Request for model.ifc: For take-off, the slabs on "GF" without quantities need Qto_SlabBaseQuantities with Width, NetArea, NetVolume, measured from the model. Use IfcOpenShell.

First a look at what the model holds.

```python
import ifcopenshell
import ifcopenshell.util.element
import ifcopenshell.util.unit

model = ifcopenshell.open("model.ifc")
print(model.schema)
for unit_type in ("LENGTHUNIT", "AREAUNIT", "VOLUMEUNIT"):
    print(unit_type, ifcopenshell.util.unit.calculate_unit_scale(model, unit_type))
storey = next(s for s in model.by_type("IfcBuildingStorey") if s.Name == "GF")
slabs = [e for e in ifcopenshell.util.element.get_decomposition(storey) if e.is_a("IfcSlab")]
for e in sorted(slabs, key=lambda e: e.id()):
    print(e.id(), e.is_a(), e.Name, list(ifcopenshell.util.element.get_psets(e, qtos_only=True)), sep=" | ")
```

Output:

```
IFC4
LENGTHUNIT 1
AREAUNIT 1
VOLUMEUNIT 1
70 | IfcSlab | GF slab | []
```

```python
import ifcopenshell
import ifcopenshell.api.pset
import ifcopenshell.geom
import ifcopenshell.util.element
import ifcopenshell.util.shape
import ifcopenshell.util.unit

model = ifcopenshell.open("model.ifc")
unit_scale = ifcopenshell.util.unit.calculate_unit_scale(model)
area_scale = ifcopenshell.util.unit.calculate_unit_scale(model, "AREAUNIT")
volume_scale = ifcopenshell.util.unit.calculate_unit_scale(model, "VOLUMEUNIT")
settings = ifcopenshell.geom.settings()

storey = next(s for s in model.by_type("IfcBuildingStorey") if s.Name == "GF")
slabs = [e for e in ifcopenshell.util.element.get_decomposition(storey) if e.is_a("IfcSlab")]

for e in sorted(slabs, key=lambda e: e.id()):
    if ifcopenshell.util.element.get_psets(e, qtos_only=True, should_inherit=False):
        continue
    # Geometry comes back in metres, in the element's own axes.
    shape = ifcopenshell.geom.create_shape(settings, e)
    values = {
        "Width": ifcopenshell.util.shape.get_z(shape.geometry) / unit_scale,
        "NetArea": ifcopenshell.util.shape.get_footprint_area(shape.geometry) / area_scale,
        "NetVolume": ifcopenshell.util.shape.get_volume(shape.geometry) / volume_scale,
    }
    qto = ifcopenshell.api.pset.add_qto(model, product=e, name="Qto_SlabBaseQuantities")
    ifcopenshell.api.pset.edit_qto(model, qto=qto, properties=values)
    print(e.id(), {k: round(v, 3) for k, v in values.items()})

model.write("model_v2.ifc")
```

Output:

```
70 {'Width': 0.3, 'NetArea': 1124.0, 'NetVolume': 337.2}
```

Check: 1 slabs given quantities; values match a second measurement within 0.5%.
